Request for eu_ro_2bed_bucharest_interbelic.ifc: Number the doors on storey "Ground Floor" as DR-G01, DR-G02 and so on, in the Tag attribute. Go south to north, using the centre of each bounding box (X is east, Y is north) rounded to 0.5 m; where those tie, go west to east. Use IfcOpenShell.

First a look at what the model holds.

```python
import ifcopenshell
import ifcopenshell.util.element
import ifcopenshell.util.placement

model = ifcopenshell.open("eu_ro_2bed_bucharest_interbelic.ifc")
print(model.schema)
storey = next(s for s in model.by_type("IfcBuildingStorey") if s.Name == "Ground Floor")
doors = [e for e in ifcopenshell.util.element.get_decomposition(storey) if e.is_a("IfcDoor")]
for e in sorted(doors, key=lambda e: e.id()):
    origin = ifcopenshell.util.placement.get_local_placement(e.ObjectPlacement)[:3, 3]
    print(e.id(), e.Tag, e.Name, origin.round(2) + 0.0, sep=" | ")
```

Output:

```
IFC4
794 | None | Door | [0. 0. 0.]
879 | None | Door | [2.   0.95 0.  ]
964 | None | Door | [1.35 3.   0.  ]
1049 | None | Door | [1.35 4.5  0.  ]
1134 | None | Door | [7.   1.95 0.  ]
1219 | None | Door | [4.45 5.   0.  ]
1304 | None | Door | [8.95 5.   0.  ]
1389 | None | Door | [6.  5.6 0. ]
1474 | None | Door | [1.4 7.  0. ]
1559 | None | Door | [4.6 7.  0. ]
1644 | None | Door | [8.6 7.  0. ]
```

```python
import ifcopenshell
import ifcopenshell.geom
import ifcopenshell.util.element
import ifcopenshell.util.shape

model = ifcopenshell.open("eu_ro_2bed_bucharest_interbelic.ifc")
settings = ifcopenshell.geom.settings()
settings.set("use-world-coords", True)


def centre(element):
    shape = ifcopenshell.geom.create_shape(settings, element)
    return ifcopenshell.util.shape.get_bbox_centroid(shape.geometry)


storey = next(s for s in model.by_type("IfcBuildingStorey") if s.Name == "Ground Floor")
doors = [e for e in ifcopenshell.util.element.get_decomposition(storey) if e.is_a("IfcDoor")]

# Insertion points can sit at a corner or the storey origin, so sort by the geometry (in metres).
centres = {e: centre(e) for e in doors}
doors.sort(key=lambda e: (round(centres[e][1] / 0.5), centres[e][0]))

for i, e in enumerate(doors, start=1):
    number = f"DR-G{i:02d}"
    e.Tag = number
    print(e.id(), number)

model.write("eu_ro_2bed_bucharest_interbelic_updated.ifc")
```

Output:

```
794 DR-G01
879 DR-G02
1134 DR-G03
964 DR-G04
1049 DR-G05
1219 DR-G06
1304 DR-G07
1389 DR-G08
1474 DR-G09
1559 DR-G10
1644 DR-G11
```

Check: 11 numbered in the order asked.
